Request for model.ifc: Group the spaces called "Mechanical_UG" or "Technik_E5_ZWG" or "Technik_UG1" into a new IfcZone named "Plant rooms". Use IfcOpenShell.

First a look at what the model holds.

```python
import ifcopenshell

model = ifcopenshell.open("model.ifc")
print(model.schema)
seen = {}
for space in model.by_type("IfcSpace"):
    seen[space.LongName] = seen.get(space.LongName, 0) + 1
for name, count in sorted(seen.items(), key=str):
    print(count, "x", name)
print("zones:", [z.Name for z in model.by_type("IfcZone")][:20])
```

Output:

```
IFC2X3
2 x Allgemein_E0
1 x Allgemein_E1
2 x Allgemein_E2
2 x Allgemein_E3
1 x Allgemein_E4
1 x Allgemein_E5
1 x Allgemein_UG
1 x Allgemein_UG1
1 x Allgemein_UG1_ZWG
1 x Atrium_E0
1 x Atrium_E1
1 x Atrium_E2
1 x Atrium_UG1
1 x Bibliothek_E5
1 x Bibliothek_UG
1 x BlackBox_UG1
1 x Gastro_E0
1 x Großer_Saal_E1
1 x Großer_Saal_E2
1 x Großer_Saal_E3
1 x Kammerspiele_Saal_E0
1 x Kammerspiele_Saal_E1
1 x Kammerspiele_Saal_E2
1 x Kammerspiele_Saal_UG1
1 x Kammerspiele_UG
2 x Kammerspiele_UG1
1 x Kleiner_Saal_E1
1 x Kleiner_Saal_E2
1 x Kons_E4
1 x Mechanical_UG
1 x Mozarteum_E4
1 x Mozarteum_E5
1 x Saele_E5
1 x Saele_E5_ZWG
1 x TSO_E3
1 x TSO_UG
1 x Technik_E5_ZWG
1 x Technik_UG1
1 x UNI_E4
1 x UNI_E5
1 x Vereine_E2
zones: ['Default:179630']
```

```python
import ifcopenshell
import ifcopenshell.api.group
import ifcopenshell.api.root

model = ifcopenshell.open("model.ifc")

names = {"Mechanical_UG", "Technik_E5_ZWG", "Technik_UG1"}
spaces = [s for s in model.by_type("IfcSpace") if s.LongName in names]

zone = ifcopenshell.api.root.create_entity(model, ifc_class="IfcZone", name="Plant rooms")
ifcopenshell.api.group.assign_group(model, products=spaces, group=zone)
print(len(spaces), "spaces in", zone.Name)

model.write("model_updated.ifc")
```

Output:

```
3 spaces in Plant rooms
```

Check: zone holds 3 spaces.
